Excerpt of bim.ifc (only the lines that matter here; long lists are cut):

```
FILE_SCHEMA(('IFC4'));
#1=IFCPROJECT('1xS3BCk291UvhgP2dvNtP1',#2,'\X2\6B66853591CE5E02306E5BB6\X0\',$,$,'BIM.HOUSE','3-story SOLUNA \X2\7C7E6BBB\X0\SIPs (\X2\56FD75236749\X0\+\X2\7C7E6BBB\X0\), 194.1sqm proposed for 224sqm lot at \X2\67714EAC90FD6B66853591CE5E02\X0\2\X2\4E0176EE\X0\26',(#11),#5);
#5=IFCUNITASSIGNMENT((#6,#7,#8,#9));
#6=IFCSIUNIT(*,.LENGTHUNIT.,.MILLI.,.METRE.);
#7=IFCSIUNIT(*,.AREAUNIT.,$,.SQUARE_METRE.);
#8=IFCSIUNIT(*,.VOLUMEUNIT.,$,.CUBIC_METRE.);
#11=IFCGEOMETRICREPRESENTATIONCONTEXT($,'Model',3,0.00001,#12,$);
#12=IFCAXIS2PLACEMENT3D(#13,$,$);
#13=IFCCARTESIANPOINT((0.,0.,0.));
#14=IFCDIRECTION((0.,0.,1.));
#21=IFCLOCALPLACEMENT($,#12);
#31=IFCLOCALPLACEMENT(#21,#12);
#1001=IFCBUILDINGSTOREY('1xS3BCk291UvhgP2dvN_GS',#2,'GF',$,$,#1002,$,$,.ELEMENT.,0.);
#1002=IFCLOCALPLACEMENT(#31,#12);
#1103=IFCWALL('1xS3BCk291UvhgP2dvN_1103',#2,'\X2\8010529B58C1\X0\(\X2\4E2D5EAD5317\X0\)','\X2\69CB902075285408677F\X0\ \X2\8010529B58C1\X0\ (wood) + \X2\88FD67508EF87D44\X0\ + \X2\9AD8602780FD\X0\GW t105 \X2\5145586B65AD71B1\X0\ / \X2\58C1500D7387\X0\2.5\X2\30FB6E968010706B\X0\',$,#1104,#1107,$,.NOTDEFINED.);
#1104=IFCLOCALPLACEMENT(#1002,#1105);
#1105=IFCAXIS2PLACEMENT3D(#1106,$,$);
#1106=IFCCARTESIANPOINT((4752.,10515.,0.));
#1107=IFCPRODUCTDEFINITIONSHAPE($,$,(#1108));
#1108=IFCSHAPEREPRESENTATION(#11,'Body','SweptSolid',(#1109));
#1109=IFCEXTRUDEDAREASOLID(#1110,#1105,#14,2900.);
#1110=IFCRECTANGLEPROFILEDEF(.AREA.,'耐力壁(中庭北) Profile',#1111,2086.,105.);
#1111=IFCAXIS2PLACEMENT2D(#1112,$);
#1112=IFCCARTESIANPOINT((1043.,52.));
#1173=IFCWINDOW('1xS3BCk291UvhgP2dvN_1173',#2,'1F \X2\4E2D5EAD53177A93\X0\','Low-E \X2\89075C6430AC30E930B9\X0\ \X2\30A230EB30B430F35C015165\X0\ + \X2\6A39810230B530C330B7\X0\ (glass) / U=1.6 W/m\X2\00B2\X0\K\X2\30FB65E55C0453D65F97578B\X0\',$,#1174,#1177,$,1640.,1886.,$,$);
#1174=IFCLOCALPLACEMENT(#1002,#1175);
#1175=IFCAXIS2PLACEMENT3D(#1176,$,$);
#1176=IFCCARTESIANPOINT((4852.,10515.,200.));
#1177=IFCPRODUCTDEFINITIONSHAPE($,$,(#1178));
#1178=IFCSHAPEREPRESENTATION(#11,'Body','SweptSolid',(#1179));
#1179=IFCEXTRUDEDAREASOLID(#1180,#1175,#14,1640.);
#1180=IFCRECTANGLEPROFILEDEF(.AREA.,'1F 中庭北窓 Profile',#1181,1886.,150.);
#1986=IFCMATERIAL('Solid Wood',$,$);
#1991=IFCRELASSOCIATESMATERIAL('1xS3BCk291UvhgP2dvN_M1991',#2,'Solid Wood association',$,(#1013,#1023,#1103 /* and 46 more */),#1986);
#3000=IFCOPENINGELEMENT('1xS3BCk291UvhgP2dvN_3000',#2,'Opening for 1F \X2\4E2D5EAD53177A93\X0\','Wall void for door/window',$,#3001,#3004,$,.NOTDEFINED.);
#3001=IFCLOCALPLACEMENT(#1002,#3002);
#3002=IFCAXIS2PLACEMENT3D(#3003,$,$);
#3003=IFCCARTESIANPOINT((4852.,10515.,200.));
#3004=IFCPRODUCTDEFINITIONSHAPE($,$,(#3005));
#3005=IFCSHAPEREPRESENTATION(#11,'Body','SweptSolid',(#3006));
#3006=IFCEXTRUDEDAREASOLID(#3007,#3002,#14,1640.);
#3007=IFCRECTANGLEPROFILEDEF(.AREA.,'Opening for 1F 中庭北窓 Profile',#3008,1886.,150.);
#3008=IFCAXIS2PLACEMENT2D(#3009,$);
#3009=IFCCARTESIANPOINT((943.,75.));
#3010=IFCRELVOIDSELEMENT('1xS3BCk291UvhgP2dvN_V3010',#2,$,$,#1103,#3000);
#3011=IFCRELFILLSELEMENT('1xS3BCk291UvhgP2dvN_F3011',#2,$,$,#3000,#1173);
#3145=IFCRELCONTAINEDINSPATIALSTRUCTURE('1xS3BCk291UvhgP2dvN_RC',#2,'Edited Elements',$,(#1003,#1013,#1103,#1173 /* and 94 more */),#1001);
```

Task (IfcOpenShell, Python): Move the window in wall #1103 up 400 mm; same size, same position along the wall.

```python
import numpy as np
import ifcopenshell
import ifcopenshell.api.geometry
import ifcopenshell.util.placement
import ifcopenshell.util.unit

model = ifcopenshell.open("bim.ifc")
unit_scale = ifcopenshell.util.unit.calculate_unit_scale(model)

window = model.by_guid("1xS3BCk291UvhgP2dvN_1173")
opening = window.FillsVoids[0].RelatingOpeningElement
dz = 0.4 / unit_scale

shift = np.array([0.0, 0.0, dz])
# The window is not placed relative to its opening, so move both.
for product in (opening, window):
    matrix = ifcopenshell.util.placement.get_local_placement(product.ObjectPlacement)
    matrix[:3, 3] += shift
    ifcopenshell.api.geometry.edit_object_placement(model, product=product, matrix=matrix, is_si=False)

print(f"moved by {dz * unit_scale:+.3f} m")

model.write("bim_rev.ifc")
```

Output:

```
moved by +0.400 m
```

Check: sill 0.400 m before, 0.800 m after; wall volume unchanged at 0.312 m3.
